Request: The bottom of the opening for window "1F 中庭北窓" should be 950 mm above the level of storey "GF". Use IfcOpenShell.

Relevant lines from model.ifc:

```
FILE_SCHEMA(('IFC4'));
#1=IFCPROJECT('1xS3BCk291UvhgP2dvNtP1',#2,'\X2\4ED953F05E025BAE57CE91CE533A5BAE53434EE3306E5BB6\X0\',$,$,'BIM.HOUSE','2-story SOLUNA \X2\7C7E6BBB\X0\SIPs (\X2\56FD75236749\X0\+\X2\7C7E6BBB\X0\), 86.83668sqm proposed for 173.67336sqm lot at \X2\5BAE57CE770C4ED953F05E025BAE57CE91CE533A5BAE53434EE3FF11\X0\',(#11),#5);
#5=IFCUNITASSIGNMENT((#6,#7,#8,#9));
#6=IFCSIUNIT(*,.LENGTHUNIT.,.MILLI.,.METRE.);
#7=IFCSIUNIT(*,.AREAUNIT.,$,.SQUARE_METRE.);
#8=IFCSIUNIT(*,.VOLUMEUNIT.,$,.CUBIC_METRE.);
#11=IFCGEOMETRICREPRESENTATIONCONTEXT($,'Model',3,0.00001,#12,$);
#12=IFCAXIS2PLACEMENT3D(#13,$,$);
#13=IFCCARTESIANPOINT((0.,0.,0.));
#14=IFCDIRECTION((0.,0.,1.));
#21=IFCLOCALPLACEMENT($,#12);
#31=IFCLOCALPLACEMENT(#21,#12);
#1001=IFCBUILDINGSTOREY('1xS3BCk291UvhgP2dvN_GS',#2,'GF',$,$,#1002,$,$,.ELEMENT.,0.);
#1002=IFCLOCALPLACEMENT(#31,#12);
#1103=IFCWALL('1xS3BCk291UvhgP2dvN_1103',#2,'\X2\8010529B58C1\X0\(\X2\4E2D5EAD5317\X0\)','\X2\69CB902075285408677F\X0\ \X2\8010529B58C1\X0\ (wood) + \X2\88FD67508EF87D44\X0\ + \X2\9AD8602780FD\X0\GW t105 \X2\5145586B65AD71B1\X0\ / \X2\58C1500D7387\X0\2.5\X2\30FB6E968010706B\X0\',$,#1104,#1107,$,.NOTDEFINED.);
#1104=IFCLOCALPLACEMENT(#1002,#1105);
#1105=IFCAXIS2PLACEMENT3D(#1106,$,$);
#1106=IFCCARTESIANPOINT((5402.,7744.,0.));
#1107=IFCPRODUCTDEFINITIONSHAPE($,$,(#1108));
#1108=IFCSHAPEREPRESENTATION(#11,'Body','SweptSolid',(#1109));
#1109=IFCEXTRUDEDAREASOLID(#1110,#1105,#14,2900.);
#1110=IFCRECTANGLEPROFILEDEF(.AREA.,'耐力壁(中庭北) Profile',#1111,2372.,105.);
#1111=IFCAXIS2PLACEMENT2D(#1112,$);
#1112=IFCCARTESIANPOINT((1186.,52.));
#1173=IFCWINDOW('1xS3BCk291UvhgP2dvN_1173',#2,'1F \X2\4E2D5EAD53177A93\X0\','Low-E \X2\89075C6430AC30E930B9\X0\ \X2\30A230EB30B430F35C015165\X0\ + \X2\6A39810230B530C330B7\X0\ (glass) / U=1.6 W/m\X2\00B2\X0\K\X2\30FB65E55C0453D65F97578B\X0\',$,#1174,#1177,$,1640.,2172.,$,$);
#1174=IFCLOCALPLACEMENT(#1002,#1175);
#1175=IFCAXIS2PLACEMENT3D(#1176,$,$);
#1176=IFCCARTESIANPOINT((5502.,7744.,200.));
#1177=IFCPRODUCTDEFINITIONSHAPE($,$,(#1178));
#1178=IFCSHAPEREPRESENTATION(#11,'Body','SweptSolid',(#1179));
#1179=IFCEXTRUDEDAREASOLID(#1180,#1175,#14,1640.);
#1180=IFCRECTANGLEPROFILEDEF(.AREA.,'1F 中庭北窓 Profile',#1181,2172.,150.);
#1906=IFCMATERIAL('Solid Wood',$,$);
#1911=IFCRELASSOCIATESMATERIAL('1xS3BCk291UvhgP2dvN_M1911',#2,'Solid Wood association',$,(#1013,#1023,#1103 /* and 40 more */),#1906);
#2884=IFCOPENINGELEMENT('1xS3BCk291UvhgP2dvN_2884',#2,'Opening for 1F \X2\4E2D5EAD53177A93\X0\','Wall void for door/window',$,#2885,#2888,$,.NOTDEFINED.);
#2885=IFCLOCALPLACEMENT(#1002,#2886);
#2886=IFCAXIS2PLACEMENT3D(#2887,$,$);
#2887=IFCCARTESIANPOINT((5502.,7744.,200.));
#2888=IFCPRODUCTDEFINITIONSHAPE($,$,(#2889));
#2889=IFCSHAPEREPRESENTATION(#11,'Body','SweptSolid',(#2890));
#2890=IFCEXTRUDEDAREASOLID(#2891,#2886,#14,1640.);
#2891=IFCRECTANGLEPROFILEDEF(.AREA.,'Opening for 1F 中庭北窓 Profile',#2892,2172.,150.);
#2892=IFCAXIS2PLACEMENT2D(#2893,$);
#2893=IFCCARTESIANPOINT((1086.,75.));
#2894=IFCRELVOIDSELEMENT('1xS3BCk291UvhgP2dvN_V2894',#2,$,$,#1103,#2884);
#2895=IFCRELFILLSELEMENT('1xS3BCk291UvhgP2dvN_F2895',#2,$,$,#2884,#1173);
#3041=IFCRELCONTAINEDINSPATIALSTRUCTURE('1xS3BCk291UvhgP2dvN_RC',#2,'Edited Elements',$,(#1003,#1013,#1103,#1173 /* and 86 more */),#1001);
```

```python
import numpy as np
import ifcopenshell
import ifcopenshell.api.geometry
import ifcopenshell.geom
import ifcopenshell.util.element
import ifcopenshell.util.placement
import ifcopenshell.util.shape
import ifcopenshell.util.unit

model = ifcopenshell.open("model.ifc")
unit_scale = ifcopenshell.util.unit.calculate_unit_scale(model)

window = model.by_guid("1xS3BCk291UvhgP2dvN_1173")
opening = window.FillsVoids[0].RelatingOpeningElement
storey = ifcopenshell.util.element.get_container(window, ifc_class="IfcBuildingStorey")
level = ifcopenshell.util.placement.get_local_placement(storey.ObjectPlacement)[2, 3]

# The opening's origin need not be at the sill, so measure its lowest point.
shape = ifcopenshell.geom.create_shape(ifcopenshell.geom.settings(), opening)
bottom = ifcopenshell.util.shape.get_shape_bottom_elevation(shape, shape.geometry) / unit_scale
dz = level + 950.0 - bottom

shift = np.array([0.0, 0.0, dz])
# The window is not placed relative to its opening, so move both.
for product in (opening, window):
    matrix = ifcopenshell.util.placement.get_local_placement(product.ObjectPlacement)
    matrix[:3, 3] += shift
    ifcopenshell.api.geometry.edit_object_placement(model, product=product, matrix=matrix, is_si=False)

print(f"moved by {dz * unit_scale:+.3f} m")

model.write("model_updated.ifc")
```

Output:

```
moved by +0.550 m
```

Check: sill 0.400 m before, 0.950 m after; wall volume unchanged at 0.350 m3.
